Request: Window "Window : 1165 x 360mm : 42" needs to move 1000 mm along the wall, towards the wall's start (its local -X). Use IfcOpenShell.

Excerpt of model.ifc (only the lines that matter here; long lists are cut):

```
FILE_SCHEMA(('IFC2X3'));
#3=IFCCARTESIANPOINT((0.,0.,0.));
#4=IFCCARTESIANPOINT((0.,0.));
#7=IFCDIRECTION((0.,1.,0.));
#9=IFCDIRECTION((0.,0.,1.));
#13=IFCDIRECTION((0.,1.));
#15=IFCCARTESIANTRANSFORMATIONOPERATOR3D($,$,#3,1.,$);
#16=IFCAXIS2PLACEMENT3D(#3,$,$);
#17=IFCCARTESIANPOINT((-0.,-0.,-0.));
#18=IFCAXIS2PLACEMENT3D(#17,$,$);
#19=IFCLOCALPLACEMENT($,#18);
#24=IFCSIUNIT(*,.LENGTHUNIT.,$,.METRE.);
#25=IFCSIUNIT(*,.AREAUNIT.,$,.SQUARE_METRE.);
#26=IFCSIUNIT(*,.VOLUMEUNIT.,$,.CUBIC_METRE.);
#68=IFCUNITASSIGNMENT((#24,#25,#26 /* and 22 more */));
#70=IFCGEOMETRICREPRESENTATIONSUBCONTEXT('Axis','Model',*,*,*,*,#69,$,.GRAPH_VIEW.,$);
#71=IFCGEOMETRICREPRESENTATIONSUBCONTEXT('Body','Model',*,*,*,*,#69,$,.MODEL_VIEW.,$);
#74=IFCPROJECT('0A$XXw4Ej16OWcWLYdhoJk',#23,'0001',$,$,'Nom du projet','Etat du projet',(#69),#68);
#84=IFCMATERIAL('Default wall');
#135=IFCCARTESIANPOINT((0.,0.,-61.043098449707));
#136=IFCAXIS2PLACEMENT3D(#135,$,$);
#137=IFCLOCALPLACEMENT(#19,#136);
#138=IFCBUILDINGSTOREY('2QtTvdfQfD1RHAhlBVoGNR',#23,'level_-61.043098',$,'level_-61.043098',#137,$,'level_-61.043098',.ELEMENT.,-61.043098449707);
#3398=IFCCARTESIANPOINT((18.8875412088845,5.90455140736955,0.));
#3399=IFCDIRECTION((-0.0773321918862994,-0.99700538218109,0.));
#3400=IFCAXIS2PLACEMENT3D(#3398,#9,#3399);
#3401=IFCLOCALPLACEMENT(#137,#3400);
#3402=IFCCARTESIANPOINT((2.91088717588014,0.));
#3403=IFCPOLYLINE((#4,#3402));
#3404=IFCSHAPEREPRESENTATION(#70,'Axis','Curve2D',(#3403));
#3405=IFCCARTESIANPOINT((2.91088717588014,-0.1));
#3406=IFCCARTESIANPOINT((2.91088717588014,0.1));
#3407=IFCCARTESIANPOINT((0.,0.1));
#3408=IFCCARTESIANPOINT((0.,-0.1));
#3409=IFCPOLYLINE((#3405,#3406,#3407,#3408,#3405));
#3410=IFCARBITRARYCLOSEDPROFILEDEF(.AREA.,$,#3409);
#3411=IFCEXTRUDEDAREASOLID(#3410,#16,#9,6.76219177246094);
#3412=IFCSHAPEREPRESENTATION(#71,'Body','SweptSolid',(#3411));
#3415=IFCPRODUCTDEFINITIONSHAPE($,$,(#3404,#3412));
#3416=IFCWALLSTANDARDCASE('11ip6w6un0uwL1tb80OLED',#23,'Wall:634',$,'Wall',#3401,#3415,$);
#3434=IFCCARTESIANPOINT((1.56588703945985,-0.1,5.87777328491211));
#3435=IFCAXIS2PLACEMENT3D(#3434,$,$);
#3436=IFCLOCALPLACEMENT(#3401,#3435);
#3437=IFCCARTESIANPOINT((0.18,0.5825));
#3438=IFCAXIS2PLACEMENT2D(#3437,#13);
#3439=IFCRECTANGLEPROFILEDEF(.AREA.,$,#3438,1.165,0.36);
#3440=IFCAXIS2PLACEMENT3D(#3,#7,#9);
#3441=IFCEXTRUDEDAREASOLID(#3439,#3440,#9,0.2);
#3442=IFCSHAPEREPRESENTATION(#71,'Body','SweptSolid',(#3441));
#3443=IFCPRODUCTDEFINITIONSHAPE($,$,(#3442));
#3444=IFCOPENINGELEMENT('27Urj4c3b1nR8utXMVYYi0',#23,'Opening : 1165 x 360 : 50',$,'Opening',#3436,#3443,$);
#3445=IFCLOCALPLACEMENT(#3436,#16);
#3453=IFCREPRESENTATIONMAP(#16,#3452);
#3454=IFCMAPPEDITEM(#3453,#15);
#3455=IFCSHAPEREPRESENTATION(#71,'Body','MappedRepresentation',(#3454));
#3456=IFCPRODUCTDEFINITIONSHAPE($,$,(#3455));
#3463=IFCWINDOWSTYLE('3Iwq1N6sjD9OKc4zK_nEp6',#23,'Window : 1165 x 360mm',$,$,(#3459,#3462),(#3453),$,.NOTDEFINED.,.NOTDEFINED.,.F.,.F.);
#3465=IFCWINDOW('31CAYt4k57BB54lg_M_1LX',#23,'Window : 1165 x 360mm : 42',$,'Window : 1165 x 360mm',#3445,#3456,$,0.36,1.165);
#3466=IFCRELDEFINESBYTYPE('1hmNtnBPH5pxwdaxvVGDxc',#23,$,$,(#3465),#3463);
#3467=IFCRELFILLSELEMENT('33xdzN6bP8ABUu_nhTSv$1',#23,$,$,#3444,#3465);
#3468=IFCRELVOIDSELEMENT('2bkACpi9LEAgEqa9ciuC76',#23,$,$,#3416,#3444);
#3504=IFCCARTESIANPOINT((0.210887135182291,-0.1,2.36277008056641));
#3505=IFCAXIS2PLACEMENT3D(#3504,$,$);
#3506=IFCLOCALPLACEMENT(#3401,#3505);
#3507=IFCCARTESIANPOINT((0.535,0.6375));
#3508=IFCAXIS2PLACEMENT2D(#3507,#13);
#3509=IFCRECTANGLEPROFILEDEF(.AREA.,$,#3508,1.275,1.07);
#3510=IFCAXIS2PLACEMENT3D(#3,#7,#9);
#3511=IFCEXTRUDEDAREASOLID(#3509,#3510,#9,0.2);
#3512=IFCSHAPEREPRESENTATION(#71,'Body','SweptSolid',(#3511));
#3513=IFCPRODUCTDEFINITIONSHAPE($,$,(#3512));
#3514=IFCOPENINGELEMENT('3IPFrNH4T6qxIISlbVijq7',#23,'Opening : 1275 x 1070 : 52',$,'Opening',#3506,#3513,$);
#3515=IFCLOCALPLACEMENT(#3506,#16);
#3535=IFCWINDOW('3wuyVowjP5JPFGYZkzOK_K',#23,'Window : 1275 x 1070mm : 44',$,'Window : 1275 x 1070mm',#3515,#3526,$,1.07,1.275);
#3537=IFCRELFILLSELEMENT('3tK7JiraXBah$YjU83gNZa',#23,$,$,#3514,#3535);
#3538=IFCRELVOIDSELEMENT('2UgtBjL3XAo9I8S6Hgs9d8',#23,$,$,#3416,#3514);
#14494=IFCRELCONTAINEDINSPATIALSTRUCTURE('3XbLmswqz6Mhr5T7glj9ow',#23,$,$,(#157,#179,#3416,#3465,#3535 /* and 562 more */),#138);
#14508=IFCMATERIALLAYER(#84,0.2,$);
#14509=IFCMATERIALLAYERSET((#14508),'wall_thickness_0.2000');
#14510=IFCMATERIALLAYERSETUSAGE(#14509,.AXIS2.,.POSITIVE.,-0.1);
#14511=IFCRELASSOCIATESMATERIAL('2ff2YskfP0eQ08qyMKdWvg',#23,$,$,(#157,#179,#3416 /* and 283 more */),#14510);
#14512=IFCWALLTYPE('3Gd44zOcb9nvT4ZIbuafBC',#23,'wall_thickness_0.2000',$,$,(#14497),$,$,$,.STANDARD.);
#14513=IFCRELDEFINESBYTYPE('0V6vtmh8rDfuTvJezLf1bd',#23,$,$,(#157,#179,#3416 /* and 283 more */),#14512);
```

```python
import ifcopenshell
import ifcopenshell.api.geometry
import ifcopenshell.util.placement
import ifcopenshell.util.unit

model = ifcopenshell.open("model.ifc")
unit_scale = ifcopenshell.util.unit.calculate_unit_scale(model)

window = model.by_id(3465)
opening = window.FillsVoids[0].RelatingOpeningElement
wall = opening.VoidsElements[0].RelatingBuildingElement

wall_matrix = ifcopenshell.util.placement.get_local_placement(wall.ObjectPlacement)
shift = wall_matrix[:3, 0] * -1 / unit_scale
before = ifcopenshell.util.placement.get_local_placement(window.ObjectPlacement)[:3, 3].copy()

# The window is placed relative to its opening, so it follows when the opening moves.
matrix = ifcopenshell.util.placement.get_local_placement(opening.ObjectPlacement)
matrix[:3, 3] += shift
ifcopenshell.api.geometry.edit_object_placement(
    model, product=opening, matrix=matrix, is_si=False, should_transform_children=True
)

after = ifcopenshell.util.placement.get_local_placement(window.ObjectPlacement)[:3, 3]
print("window moved by", (after - before).round(3) + 0.0)

model.write("model-out.ifc")
```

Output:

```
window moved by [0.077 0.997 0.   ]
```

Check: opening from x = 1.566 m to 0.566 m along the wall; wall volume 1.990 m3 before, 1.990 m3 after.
